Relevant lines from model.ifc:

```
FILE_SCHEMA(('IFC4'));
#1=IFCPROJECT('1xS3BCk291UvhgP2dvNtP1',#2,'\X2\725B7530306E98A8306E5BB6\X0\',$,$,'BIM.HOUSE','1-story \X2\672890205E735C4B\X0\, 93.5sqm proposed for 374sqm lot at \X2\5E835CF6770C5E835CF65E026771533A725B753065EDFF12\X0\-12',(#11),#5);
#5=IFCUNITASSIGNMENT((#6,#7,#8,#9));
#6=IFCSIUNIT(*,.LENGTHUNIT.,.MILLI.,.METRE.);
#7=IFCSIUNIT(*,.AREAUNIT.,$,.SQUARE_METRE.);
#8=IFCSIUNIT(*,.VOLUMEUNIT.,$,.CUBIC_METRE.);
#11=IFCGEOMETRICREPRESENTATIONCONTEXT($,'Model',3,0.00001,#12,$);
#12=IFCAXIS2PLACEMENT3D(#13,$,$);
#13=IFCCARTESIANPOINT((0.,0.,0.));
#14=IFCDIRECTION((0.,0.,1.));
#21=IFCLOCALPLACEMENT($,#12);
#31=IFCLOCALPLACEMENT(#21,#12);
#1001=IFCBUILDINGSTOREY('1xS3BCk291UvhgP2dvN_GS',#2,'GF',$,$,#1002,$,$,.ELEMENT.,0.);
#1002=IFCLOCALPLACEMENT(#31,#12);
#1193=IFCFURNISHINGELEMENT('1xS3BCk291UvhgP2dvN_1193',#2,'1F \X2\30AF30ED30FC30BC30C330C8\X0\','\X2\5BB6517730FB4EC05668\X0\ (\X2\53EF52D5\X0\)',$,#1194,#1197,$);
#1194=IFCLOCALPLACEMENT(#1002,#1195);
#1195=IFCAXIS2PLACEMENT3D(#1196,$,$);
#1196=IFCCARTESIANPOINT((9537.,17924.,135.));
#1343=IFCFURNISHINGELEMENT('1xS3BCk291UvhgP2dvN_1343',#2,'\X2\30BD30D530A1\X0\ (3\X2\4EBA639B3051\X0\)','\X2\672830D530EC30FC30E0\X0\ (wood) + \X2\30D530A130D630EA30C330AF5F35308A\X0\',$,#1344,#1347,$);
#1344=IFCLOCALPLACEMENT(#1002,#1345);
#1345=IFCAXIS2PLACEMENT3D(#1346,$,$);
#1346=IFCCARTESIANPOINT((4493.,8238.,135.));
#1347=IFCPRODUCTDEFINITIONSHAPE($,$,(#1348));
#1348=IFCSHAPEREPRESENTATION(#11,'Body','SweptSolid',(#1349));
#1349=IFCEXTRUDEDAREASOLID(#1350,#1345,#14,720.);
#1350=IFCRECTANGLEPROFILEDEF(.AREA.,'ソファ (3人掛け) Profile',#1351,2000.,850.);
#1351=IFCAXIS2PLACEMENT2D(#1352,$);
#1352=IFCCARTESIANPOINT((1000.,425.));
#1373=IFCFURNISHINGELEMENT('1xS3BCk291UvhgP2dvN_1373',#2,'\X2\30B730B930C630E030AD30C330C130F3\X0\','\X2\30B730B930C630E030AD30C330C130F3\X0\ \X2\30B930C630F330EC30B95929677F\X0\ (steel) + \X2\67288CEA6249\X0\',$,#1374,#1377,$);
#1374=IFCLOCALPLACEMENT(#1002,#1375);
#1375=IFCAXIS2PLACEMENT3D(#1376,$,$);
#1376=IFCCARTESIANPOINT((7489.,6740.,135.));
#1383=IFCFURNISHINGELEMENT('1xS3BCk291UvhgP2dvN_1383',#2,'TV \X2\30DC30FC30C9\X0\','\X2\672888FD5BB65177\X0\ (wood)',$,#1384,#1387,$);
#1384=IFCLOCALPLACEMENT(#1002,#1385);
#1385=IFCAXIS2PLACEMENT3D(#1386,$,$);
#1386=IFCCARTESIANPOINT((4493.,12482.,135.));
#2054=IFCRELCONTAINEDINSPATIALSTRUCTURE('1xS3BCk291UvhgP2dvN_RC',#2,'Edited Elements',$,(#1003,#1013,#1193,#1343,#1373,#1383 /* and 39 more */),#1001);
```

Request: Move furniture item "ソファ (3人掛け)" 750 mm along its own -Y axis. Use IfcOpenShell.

```python
import ifcopenshell
import ifcopenshell.api.geometry
import ifcopenshell.util.placement

model = ifcopenshell.open("model.ifc")

item = model.by_guid("1xS3BCk291UvhgP2dvN_1343")
matrix = ifcopenshell.util.placement.get_local_placement(item.ObjectPlacement)
matrix[:3, 3] -= matrix[:3, 1] * 750.0
ifcopenshell.api.geometry.edit_object_placement(model, product=item, matrix=matrix, is_si=False)

print(ifcopenshell.util.placement.get_local_placement(item.ObjectPlacement).round(3) + 0.0)

model.write("model-out.ifc")
```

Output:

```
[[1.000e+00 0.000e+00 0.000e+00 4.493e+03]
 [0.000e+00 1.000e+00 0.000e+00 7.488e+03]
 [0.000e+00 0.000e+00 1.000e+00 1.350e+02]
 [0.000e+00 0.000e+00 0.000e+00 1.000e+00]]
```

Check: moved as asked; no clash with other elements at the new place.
